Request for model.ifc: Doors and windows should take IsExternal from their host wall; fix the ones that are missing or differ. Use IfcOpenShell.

First a look at what the model holds.

```python
import ifcopenshell
import ifcopenshell.util.element

model = ifcopenshell.open("model.ifc")
print(model.schema)
seen = {}
for e in model.by_type("IfcDoor") + model.by_type("IfcWindow"):
    if not e.FillsVoids:
        continue
    host = e.FillsVoids[0].RelatingOpeningElement.VoidsElements[0].RelatingBuildingElement
    own = ifcopenshell.util.element.get_pset(e, f"Pset_{e.is_a()[3:].removesuffix('StandardCase')}Common", "IsExternal")
    wall = ifcopenshell.util.element.get_pset(host, "Pset_WallCommon", "IsExternal")
    seen[e.is_a(), own, wall] = seen.get((e.is_a(), own, wall), 0) + 1
for (cls, own, wall), count in sorted(seen.items(), key=str):
    print(count, cls, "IsExternal:", own, "| host wall:", wall)
```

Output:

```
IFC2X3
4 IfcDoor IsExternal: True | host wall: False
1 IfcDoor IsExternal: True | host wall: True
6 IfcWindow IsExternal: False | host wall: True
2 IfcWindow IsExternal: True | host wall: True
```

```python
import ifcopenshell
import ifcopenshell.api.pset
import ifcopenshell.util.element

model = ifcopenshell.open("model.ifc")

count = 0
for ifc_class, pset_name in (("IfcDoor", "Pset_DoorCommon"), ("IfcWindow", "Pset_WindowCommon")):
    for e in model.by_type(ifc_class):
        if not e.FillsVoids:
            continue
        host = e.FillsVoids[0].RelatingOpeningElement.VoidsElements[0].RelatingBuildingElement
        external = ifcopenshell.util.element.get_pset(host, "Pset_WallCommon", "IsExternal")
        if external is None or ifcopenshell.util.element.get_pset(e, pset_name, "IsExternal") == external:
            continue
        pset = ifcopenshell.api.pset.add_pset(model, product=e, name=pset_name)
        ifcopenshell.api.pset.edit_pset(model, pset=pset, properties={"IsExternal": external})
        count += 1

print(count, "updated")

model.write("model_rev.ifc")
```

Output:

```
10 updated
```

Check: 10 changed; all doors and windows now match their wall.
